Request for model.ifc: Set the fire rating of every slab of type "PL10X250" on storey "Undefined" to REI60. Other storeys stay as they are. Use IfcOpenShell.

First a look at what the model holds.

```python
import ifcopenshell
import ifcopenshell.util.element

model = ifcopenshell.open("model.ifc")
print(model.schema)
storey = next(s for s in model.by_type("IfcBuildingStorey") if s.Name == "Undefined")
slabs = [e for e in ifcopenshell.util.element.get_decomposition(storey) if e.is_a("IfcSlab")]
seen = {}
for e in slabs:
    element_type = ifcopenshell.util.element.get_type(e)
    key = (element_type.Name if element_type != e and element_type else None, ifcopenshell.util.element.get_pset(e, "Pset_SlabCommon", "FireRating"))
    seen[key] = seen.get(key, 0) + 1
for (name, value), count in sorted(seen.items(), key=str):
    print(count, "x", name, "|", value)
```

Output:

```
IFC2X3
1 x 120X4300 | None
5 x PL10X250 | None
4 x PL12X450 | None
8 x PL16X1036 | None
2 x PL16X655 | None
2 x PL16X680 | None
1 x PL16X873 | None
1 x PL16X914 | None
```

```python
import ifcopenshell
import ifcopenshell.api.pset
import ifcopenshell.util.element

model = ifcopenshell.open("model.ifc")

storey = next(s for s in model.by_type("IfcBuildingStorey") if s.Name == "Undefined")
slabs = [e for e in ifcopenshell.util.element.get_decomposition(storey) if e.is_a("IfcSlab")]

count = 0
for e in slabs:
    element_type = ifcopenshell.util.element.get_type(e)
    if element_type in (None, e) or element_type.Name != "PL10X250":
        continue
    found = ifcopenshell.util.element.get_pset(e, "Pset_SlabCommon", should_inherit=False)
    if found:
        pset = model.by_id(found["id"])
        if len(ifcopenshell.util.element.get_elements_by_pset(pset)) > 1:
            pset = ifcopenshell.api.pset.unshare_pset(model, products=[e], pset=pset)[0]
    else:
        pset = ifcopenshell.api.pset.add_pset(model, product=e, name="Pset_SlabCommon")
    ifcopenshell.api.pset.edit_pset(model, pset=pset, properties={"FireRating": "REI60"})
    count += 1

print(count, "slabs updated")

model.write("model_rev.ifc")
```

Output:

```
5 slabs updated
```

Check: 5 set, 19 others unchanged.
